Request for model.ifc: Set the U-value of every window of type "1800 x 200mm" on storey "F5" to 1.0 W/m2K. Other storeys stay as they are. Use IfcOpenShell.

First a look at what the model holds.

```python
import ifcopenshell
import ifcopenshell.util.element

model = ifcopenshell.open("model.ifc")
print(model.schema)
storey = next(s for s in model.by_type("IfcBuildingStorey") if s.Name == "F5")
windows = [e for e in ifcopenshell.util.element.get_decomposition(storey) if e.is_a("IfcWindow")]
seen = {}
for e in windows:
    element_type = ifcopenshell.util.element.get_type(e)
    key = (element_type.Name if element_type != e and element_type else None, ifcopenshell.util.element.get_pset(e, "Pset_WindowCommon", "ThermalTransmittance"))
    seen[key] = seen.get(key, 0) + 1
for (name, value), count in sorted(seen.items(), key=str):
    print(count, "x", name, "|", value)
```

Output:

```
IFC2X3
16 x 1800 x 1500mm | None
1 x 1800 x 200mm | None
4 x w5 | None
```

```python
import ifcopenshell
import ifcopenshell.api.pset
import ifcopenshell.util.element

model = ifcopenshell.open("model.ifc")

storey = next(s for s in model.by_type("IfcBuildingStorey") if s.Name == "F5")
windows = [e for e in ifcopenshell.util.element.get_decomposition(storey) if e.is_a("IfcWindow")]

count = 0
for e in windows:
    element_type = ifcopenshell.util.element.get_type(e)
    if element_type in (None, e) or element_type.Name != "1800 x 200mm":
        continue
    # add_pset returns the element's existing set when there is one.
    pset = ifcopenshell.api.pset.add_pset(model, product=e, name="Pset_WindowCommon")
    ifcopenshell.api.pset.edit_pset(model, pset=pset, properties={"ThermalTransmittance": 1.0})
    count += 1

print(count, "windows updated")

model.write("model_v2.ifc")
```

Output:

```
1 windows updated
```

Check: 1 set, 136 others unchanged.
